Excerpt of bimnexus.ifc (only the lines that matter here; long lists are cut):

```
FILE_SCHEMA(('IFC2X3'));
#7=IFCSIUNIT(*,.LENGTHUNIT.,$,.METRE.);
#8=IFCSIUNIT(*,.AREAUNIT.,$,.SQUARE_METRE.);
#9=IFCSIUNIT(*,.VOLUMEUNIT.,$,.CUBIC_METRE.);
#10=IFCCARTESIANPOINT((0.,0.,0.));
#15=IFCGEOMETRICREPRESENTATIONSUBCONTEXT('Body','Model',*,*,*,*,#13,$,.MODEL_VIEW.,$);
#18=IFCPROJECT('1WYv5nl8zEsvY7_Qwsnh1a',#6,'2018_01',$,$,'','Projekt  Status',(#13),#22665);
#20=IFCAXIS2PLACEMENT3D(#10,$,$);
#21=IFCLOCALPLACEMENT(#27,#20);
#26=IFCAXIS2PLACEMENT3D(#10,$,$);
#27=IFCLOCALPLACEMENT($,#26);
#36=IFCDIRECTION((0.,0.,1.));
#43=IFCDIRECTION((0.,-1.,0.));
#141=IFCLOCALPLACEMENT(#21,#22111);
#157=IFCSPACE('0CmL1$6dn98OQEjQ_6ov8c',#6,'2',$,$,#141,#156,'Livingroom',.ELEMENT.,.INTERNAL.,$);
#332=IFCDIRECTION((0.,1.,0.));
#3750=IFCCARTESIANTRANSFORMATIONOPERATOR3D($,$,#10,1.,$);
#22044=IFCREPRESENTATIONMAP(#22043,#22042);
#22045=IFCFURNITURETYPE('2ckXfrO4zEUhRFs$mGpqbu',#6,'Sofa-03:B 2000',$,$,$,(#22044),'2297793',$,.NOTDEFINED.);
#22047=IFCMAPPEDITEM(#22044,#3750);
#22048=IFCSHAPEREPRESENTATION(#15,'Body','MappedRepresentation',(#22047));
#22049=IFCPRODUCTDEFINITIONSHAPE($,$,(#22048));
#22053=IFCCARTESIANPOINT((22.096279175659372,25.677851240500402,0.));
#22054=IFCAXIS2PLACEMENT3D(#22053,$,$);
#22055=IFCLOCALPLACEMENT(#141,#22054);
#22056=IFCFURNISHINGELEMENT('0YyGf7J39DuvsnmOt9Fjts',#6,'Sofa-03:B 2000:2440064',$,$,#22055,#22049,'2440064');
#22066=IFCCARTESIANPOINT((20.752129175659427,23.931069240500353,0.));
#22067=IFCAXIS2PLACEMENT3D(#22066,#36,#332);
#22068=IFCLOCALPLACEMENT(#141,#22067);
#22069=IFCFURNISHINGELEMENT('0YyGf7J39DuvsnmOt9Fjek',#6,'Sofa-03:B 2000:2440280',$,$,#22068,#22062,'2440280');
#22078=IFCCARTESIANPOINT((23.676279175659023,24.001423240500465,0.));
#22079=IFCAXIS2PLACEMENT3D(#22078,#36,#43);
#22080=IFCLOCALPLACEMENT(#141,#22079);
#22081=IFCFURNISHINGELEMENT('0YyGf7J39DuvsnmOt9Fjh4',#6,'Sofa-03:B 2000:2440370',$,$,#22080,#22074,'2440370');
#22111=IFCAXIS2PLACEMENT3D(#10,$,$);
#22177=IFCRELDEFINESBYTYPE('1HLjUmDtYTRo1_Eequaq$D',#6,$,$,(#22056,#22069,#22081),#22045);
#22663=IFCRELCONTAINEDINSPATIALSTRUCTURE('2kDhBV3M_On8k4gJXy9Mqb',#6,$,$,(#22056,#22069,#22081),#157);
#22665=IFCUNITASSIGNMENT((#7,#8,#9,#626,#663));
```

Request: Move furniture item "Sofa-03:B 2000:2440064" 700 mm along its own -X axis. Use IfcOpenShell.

```python
import ifcopenshell
import ifcopenshell.api.geometry
import ifcopenshell.util.placement
import ifcopenshell.util.unit

model = ifcopenshell.open("bimnexus.ifc")
unit_scale = ifcopenshell.util.unit.calculate_unit_scale(model)

item = model.by_guid("0YyGf7J39DuvsnmOt9Fjts")
matrix = ifcopenshell.util.placement.get_local_placement(item.ObjectPlacement)
matrix[:3, 3] -= matrix[:3, 0] * 0.7 / unit_scale
ifcopenshell.api.geometry.edit_object_placement(model, product=item, matrix=matrix, is_si=False)

print(ifcopenshell.util.placement.get_local_placement(item.ObjectPlacement).round(3) + 0.0)

model.write("bimnexus_v2.ifc")
```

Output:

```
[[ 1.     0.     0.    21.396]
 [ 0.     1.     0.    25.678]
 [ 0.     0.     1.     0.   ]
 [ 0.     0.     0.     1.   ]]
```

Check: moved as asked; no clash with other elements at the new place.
